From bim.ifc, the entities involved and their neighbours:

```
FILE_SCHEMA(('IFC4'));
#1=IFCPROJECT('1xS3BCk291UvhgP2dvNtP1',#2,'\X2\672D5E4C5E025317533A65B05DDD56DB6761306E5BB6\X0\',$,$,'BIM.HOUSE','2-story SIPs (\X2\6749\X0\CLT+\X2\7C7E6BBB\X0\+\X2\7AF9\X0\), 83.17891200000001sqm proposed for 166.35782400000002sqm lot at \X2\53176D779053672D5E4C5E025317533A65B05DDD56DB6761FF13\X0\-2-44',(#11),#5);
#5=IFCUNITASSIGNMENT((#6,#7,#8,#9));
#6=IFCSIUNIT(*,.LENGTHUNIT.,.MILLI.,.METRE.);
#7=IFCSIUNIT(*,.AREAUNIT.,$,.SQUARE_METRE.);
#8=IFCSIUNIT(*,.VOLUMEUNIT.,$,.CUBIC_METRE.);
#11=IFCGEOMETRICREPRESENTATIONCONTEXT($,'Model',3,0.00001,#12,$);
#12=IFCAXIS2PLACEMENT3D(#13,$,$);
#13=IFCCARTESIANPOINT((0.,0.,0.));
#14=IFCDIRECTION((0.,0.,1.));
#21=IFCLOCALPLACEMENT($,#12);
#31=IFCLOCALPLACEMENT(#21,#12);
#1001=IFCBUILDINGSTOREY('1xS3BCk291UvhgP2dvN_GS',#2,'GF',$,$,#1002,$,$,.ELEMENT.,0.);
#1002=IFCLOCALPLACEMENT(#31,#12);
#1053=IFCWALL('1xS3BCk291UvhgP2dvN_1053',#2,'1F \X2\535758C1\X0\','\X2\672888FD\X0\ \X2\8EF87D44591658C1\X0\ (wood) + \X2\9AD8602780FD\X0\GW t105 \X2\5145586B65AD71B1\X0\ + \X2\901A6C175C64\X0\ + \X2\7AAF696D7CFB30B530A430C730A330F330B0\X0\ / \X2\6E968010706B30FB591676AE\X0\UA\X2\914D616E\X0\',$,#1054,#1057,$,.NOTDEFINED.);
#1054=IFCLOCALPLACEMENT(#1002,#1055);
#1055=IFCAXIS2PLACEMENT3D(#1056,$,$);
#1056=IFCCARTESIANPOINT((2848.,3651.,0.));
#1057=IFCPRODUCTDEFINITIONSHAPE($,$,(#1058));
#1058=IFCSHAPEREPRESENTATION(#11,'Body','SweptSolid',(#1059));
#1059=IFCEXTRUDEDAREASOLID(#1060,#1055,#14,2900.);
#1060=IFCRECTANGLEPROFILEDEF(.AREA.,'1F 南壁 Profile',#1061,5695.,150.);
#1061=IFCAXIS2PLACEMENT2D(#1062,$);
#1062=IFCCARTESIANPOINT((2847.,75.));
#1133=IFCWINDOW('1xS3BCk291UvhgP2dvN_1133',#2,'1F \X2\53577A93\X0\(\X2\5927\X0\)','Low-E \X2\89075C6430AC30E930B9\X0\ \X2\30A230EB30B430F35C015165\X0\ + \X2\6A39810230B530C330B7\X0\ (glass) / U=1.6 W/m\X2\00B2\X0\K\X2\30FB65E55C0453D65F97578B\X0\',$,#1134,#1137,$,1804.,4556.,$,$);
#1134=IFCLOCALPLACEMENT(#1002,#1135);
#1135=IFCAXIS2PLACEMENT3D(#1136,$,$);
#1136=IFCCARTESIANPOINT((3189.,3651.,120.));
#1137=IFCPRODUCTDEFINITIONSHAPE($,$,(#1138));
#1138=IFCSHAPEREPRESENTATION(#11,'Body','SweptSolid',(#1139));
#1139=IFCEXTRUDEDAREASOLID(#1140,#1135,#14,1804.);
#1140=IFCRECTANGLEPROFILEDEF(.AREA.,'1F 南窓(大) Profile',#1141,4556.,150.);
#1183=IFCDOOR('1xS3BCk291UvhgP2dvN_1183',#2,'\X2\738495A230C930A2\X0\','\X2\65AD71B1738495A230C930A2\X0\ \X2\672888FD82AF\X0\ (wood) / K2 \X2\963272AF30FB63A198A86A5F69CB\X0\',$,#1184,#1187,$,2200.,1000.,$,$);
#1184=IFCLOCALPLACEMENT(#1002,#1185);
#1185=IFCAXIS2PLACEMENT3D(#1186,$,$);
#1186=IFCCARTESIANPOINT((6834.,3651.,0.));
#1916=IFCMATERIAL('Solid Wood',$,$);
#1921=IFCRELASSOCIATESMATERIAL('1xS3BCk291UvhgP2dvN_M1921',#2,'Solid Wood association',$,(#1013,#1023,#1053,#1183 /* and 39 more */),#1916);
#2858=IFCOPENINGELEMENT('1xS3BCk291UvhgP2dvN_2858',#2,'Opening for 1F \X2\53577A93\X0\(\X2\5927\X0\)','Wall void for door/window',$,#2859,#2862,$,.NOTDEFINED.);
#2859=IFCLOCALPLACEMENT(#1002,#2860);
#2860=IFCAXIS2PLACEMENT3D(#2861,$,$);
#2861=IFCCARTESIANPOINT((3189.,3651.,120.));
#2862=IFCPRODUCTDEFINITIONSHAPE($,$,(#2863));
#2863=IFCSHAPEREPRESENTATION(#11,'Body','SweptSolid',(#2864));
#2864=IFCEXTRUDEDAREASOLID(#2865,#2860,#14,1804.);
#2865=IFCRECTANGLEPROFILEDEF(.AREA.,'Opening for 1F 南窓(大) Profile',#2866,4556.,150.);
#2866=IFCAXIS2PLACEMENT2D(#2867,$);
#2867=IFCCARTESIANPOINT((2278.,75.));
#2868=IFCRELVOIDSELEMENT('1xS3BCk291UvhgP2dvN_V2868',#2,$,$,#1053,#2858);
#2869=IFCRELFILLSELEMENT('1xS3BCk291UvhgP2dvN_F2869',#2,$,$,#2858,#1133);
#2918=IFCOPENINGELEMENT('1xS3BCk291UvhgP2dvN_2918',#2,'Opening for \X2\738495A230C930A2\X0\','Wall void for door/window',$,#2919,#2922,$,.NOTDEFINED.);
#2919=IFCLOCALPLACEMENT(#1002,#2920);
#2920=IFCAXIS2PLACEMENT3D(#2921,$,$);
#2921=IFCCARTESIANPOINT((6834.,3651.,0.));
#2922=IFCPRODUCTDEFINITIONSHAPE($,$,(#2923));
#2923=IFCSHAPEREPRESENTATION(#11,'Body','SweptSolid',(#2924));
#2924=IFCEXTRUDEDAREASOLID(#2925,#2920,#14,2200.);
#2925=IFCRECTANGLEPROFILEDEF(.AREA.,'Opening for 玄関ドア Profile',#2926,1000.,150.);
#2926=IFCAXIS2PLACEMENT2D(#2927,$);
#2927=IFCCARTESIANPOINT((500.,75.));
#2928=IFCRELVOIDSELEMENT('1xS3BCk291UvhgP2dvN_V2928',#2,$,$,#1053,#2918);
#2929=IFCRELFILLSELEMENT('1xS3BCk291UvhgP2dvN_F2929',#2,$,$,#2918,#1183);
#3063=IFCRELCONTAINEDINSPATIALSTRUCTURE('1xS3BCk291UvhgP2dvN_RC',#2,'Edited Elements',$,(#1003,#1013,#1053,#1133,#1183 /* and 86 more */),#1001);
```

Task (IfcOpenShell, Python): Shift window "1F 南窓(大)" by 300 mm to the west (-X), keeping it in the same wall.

```python
import ifcopenshell
import ifcopenshell.api.geometry
import ifcopenshell.util.placement

model = ifcopenshell.open("bim.ifc")

window = model.by_id(1133)
opening = window.FillsVoids[0].RelatingOpeningElement
wall = opening.VoidsElements[0].RelatingBuildingElement

wall_matrix = ifcopenshell.util.placement.get_local_placement(wall.ObjectPlacement)
shift = wall_matrix[:3, 0] * -300.0
before = ifcopenshell.util.placement.get_local_placement(window.ObjectPlacement)[:3, 3].copy()

# The window is not placed relative to its opening, so move both.
for product in (opening, window):
    matrix = ifcopenshell.util.placement.get_local_placement(product.ObjectPlacement)
    matrix[:3, 3] += shift
    ifcopenshell.api.geometry.edit_object_placement(model, product=product, matrix=matrix, is_si=False)

after = ifcopenshell.util.placement.get_local_placement(window.ObjectPlacement)[:3, 3]
print("window moved by", (after - before).round(3) + 0.0)

model.write("bim-out.ifc")
```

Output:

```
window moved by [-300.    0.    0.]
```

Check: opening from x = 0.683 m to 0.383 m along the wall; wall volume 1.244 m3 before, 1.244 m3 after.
